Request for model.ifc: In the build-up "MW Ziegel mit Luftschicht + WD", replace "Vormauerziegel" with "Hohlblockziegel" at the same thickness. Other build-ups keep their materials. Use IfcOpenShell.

First a look at what the model holds.

```python
import ifcopenshell
import ifcopenshell.util.element

model = ifcopenshell.open("model.ifc")
print(model.schema)
for layer_set in model.by_type("IfcMaterialLayerSet"):
    if layer_set.LayerSetName == "MW Ziegel mit Luftschicht + WD":
        for layer in layer_set.MaterialLayers:
            print(layer.id(), layer.Material and layer.Material.Name, layer.LayerThickness, sep=" | ")
        print(len(ifcopenshell.util.element.get_elements_by_material(model, layer_set)), "elements and types use it")
print(sorted(m.Name for m in model.by_type("IfcMaterial") if m.Name)[:60])
```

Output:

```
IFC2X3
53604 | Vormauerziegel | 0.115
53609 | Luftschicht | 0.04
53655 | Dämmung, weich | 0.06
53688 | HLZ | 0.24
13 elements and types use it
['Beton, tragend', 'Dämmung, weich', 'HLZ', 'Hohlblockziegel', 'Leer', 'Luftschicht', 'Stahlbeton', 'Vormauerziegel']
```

```python
import ifcopenshell
import ifcopenshell.api.material

model = ifcopenshell.open("model.ifc")

layer_set = next(s for s in model.by_type("IfcMaterialLayerSet") if s.LayerSetName == "MW Ziegel mit Luftschicht + WD")
layer = next(l for l in layer_set.MaterialLayers if l.Material and l.Material.Name == "Vormauerziegel")
material = next(m for m in model.by_type("IfcMaterial") if m.Name == "Hohlblockziegel")

# Point this one layer at the other material; renaming the old one would change it everywhere.
ifcopenshell.api.material.edit_layer(model, layer=layer, attributes={}, material=material)

print([l.Material.Name if l.Material else None for l in layer_set.MaterialLayers])

model.write("model_edited.ifc")
```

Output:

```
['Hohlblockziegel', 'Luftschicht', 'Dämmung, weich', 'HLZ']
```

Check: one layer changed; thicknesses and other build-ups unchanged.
